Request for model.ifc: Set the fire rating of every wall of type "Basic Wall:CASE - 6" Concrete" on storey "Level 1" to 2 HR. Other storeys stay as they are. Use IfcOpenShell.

First a look at what the model holds.

```python
import ifcopenshell
import ifcopenshell.util.element

model = ifcopenshell.open("model.ifc")
print(model.schema)
storey = next(s for s in model.by_type("IfcBuildingStorey") if s.Name == "Level 1")
walls = [e for e in ifcopenshell.util.element.get_decomposition(storey) if e.is_a("IfcWall")]
seen = {}
for e in walls:
    element_type = ifcopenshell.util.element.get_type(e)
    key = (element_type.Name if element_type != e and element_type else None, ifcopenshell.util.element.get_pset(e, "Pset_WallCommon", "FireRating"))
    seen[key] = seen.get(key, 0) + 1
for (name, value), count in sorted(seen.items(), key=str):
    print(count, "x", name, "|", value)
```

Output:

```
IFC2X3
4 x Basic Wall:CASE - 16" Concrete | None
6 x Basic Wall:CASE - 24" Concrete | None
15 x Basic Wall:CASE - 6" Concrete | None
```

```python
import ifcopenshell
import ifcopenshell.api.pset
import ifcopenshell.util.element

model = ifcopenshell.open("model.ifc")

storey = next(s for s in model.by_type("IfcBuildingStorey") if s.Name == "Level 1")
walls = [e for e in ifcopenshell.util.element.get_decomposition(storey) if e.is_a("IfcWall")]

count = 0
for e in walls:
    element_type = ifcopenshell.util.element.get_type(e)
    if element_type in (None, e) or element_type.Name != 'Basic Wall:CASE - 6" Concrete':
        continue
    # add_pset returns the element's existing set when there is one.
    pset = ifcopenshell.api.pset.add_pset(model, product=e, name="Pset_WallCommon")
    ifcopenshell.api.pset.edit_pset(model, pset=pset, properties={"FireRating": "2 HR"})
    count += 1

print(count, "walls updated")

model.write("model_rev.ifc")
```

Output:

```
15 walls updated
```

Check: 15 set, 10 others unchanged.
